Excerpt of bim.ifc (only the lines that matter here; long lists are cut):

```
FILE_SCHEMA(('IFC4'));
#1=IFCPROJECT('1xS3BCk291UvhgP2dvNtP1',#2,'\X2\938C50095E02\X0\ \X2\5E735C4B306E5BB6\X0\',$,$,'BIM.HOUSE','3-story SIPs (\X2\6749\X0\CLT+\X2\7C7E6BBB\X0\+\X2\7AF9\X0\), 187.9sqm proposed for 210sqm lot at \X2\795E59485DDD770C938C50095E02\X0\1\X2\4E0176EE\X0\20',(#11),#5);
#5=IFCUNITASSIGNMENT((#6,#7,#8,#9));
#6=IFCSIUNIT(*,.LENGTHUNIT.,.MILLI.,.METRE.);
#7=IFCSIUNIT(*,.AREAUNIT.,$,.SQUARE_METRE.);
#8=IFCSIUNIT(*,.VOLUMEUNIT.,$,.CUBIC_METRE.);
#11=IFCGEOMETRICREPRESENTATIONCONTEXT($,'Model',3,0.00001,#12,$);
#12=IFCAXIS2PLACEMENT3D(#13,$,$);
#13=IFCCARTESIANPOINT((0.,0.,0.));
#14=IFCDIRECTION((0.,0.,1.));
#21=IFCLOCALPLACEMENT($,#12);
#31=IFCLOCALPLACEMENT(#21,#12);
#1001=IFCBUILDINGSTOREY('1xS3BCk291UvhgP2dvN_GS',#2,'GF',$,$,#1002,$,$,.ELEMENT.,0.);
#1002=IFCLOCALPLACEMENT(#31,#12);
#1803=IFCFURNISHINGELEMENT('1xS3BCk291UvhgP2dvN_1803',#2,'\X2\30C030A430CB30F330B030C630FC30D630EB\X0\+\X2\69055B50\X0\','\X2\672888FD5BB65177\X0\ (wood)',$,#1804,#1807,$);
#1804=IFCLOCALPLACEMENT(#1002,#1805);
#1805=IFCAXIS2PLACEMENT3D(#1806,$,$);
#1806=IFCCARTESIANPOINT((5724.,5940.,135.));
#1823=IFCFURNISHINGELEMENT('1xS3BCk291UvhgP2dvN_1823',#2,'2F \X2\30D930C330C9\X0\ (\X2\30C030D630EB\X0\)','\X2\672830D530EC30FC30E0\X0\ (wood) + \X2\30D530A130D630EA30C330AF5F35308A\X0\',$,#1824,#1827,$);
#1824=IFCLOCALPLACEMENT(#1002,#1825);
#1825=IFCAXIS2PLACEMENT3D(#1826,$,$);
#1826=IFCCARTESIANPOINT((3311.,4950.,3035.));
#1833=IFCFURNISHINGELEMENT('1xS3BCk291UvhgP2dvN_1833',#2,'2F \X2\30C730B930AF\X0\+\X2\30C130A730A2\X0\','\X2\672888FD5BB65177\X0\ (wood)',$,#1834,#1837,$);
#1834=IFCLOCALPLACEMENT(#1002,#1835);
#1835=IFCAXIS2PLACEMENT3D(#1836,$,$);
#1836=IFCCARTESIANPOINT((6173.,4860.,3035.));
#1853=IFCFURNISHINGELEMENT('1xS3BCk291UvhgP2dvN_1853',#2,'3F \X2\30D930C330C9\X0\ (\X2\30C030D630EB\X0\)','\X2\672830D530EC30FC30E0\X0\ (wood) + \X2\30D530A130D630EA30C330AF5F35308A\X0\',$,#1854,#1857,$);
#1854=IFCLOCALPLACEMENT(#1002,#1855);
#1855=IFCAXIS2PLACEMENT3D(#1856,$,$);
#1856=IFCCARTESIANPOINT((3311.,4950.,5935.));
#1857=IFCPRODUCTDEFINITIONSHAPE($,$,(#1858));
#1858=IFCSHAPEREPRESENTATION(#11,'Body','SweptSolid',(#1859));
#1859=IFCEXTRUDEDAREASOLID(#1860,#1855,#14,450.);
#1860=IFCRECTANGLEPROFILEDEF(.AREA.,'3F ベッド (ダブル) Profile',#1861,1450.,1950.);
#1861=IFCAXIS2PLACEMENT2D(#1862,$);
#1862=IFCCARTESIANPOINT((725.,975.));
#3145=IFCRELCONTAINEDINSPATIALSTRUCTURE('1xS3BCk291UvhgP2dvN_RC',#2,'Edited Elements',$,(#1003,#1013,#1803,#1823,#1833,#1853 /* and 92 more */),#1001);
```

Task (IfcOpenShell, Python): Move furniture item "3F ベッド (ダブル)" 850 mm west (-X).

```python
import ifcopenshell
import ifcopenshell.api.geometry
import ifcopenshell.util.placement

model = ifcopenshell.open("bim.ifc")

item = model.by_id(1853)
matrix = ifcopenshell.util.placement.get_local_placement(item.ObjectPlacement)
matrix[0, 3] -= 850.0
ifcopenshell.api.geometry.edit_object_placement(model, product=item, matrix=matrix, is_si=False)

print(ifcopenshell.util.placement.get_local_placement(item.ObjectPlacement).round(3) + 0.0)

model.write("bim_updated.ifc")
```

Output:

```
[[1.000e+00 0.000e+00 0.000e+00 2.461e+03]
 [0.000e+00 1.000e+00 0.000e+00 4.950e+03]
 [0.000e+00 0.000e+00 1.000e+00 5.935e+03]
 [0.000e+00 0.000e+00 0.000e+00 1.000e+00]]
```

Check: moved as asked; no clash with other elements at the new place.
